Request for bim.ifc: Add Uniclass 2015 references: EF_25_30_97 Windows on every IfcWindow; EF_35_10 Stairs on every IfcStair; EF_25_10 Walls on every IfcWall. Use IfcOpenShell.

First a look at what the model holds.

```python
import ifcopenshell

model = ifcopenshell.open("bim.ifc")
print(model.schema)
print("classifications:", [c.Name for c in model.by_type("IfcClassification")])
for ifc_class in ("IfcDoor", "IfcRoof", "IfcStair", "IfcWall", "IfcWindow"):
    print(ifc_class, len(model.by_type(ifc_class)))
```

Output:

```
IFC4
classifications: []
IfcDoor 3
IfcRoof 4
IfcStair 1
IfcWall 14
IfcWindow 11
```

```python
import ifcopenshell
import ifcopenshell.api.classification

model = ifcopenshell.open("bim.ifc")

system = ifcopenshell.api.classification.add_classification(model, classification="Uniclass 2015")

codes = {
    "IfcWindow": ("EF_25_30_97", "Windows"),
    "IfcStair": ("EF_35_10", "Stairs"),
    "IfcWall": ("EF_25_10", "Walls"),
}
for ifc_class, (code, name) in codes.items():
    products = model.by_type(ifc_class)
    ifcopenshell.api.classification.add_reference(
        model, products=products, classification=system, identification=code, name=name
    )
    print(code, len(products))

model.write("bim_rev.ifc")
```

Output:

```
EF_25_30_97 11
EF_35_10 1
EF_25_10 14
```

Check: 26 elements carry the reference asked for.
